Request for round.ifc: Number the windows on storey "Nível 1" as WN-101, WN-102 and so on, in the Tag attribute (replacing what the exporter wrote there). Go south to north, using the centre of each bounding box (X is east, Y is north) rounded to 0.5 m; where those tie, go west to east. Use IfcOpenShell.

First a look at what the model holds.

```python
import ifcopenshell
import ifcopenshell.util.element
import ifcopenshell.util.placement

model = ifcopenshell.open("round.ifc")
print(model.schema)
storey = next(s for s in model.by_type("IfcBuildingStorey") if s.Name == "Nível 1")
windows = [e for e in ifcopenshell.util.element.get_decomposition(storey) if e.is_a("IfcWindow")]
for e in sorted(windows, key=lambda e: e.id()):
    origin = ifcopenshell.util.placement.get_local_placement(e.ObjectPlacement)[:3, 3]
    print(e.id(), e.Tag, e.Name, origin.round(2) + 0.0, sep=" | ")
```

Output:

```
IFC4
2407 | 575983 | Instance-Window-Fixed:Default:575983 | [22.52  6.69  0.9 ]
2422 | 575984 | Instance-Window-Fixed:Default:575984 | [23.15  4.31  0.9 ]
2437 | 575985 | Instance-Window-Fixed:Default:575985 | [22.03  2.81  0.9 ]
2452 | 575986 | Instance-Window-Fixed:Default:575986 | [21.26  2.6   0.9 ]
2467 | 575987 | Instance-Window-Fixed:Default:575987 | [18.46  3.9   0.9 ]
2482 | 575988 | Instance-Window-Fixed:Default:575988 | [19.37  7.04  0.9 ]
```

```python
import ifcopenshell
import ifcopenshell.geom
import ifcopenshell.util.element
import ifcopenshell.util.shape

model = ifcopenshell.open("round.ifc")
settings = ifcopenshell.geom.settings()
settings.set("use-world-coords", True)


def centre(element):
    shape = ifcopenshell.geom.create_shape(settings, element)
    return ifcopenshell.util.shape.get_bbox_centroid(shape.geometry)


storey = next(s for s in model.by_type("IfcBuildingStorey") if s.Name == "Nível 1")
windows = [e for e in ifcopenshell.util.element.get_decomposition(storey) if e.is_a("IfcWindow")]

# Insertion points can sit at a corner or the storey origin, so sort by the geometry (in metres).
centres = {e: centre(e) for e in windows}
windows.sort(key=lambda e: (round(centres[e][1] / 0.5), centres[e][0]))

for i, e in enumerate(windows, start=1):
    number = f"WN-1{i:02d}"
    e.Tag = number
    print(e.id(), number)

model.write("round_v2.ifc")
```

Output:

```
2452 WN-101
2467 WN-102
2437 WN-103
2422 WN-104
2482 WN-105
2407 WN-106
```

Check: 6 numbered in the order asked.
